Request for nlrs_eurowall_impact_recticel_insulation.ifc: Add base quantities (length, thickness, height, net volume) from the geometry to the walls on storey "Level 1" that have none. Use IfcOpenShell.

First a look at what the model holds.

```python
import ifcopenshell
import ifcopenshell.util.element
import ifcopenshell.util.unit

model = ifcopenshell.open("nlrs_eurowall_impact_recticel_insulation.ifc")
print(model.schema)
for unit_type in ("LENGTHUNIT", "AREAUNIT", "VOLUMEUNIT"):
    print(unit_type, ifcopenshell.util.unit.calculate_unit_scale(model, unit_type))
storey = next(s for s in model.by_type("IfcBuildingStorey") if s.Name == "Level 1")
walls = [e for e in ifcopenshell.util.element.get_decomposition(storey) if e.is_a("IfcWall")]
for e in sorted(walls, key=lambda e: e.id()):
    print(e.id(), e.is_a(), e.Name, list(ifcopenshell.util.element.get_psets(e, qtos_only=True)), sep=" | ")
```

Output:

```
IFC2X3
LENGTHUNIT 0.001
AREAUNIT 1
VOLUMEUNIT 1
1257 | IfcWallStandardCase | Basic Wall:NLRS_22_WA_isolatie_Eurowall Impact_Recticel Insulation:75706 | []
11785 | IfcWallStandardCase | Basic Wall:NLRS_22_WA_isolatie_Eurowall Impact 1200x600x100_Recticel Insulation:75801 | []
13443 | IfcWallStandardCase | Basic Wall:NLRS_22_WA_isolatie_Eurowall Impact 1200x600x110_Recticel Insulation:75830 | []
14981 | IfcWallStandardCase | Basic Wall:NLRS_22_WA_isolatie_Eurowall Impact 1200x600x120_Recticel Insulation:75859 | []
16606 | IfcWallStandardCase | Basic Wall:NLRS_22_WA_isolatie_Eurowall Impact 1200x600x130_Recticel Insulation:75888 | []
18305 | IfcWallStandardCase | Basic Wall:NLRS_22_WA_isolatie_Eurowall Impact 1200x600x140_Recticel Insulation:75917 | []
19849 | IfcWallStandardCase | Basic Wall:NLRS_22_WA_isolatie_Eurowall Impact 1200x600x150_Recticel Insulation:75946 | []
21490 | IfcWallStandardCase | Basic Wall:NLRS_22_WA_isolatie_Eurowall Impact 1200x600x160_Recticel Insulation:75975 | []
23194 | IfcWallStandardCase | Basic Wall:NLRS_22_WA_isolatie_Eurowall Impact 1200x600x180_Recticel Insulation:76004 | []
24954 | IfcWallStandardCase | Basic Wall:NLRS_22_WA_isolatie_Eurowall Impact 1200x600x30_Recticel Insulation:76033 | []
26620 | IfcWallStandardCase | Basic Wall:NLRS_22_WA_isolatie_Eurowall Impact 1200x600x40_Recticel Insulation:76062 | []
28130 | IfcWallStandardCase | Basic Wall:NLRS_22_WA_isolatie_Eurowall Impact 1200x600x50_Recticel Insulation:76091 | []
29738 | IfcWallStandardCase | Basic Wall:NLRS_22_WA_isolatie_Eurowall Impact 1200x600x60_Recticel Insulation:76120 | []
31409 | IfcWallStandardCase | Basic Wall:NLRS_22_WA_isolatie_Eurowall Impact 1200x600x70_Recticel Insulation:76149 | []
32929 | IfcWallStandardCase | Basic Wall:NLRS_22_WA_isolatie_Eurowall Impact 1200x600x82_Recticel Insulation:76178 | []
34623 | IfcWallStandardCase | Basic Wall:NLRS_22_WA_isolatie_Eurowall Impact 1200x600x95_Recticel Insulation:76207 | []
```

```python
import ifcopenshell
import ifcopenshell.api.pset
import ifcopenshell.geom
import ifcopenshell.util.element
import ifcopenshell.util.shape
import ifcopenshell.util.unit

model = ifcopenshell.open("nlrs_eurowall_impact_recticel_insulation.ifc")
unit_scale = ifcopenshell.util.unit.calculate_unit_scale(model)
volume_scale = ifcopenshell.util.unit.calculate_unit_scale(model, "VOLUMEUNIT")
settings = ifcopenshell.geom.settings()

storey = next(s for s in model.by_type("IfcBuildingStorey") if s.Name == "Level 1")
walls = [e for e in ifcopenshell.util.element.get_decomposition(storey) if e.is_a("IfcWall")]

for e in sorted(walls, key=lambda e: e.id()):
    if ifcopenshell.util.element.get_psets(e, qtos_only=True, should_inherit=False):
        continue
    # Geometry comes back in metres, in the element's own axes.
    shape = ifcopenshell.geom.create_shape(settings, e)
    values = {
        "Length": ifcopenshell.util.shape.get_x(shape.geometry) / unit_scale,
        "Width": ifcopenshell.util.shape.get_y(shape.geometry) / unit_scale,
        "Height": ifcopenshell.util.shape.get_z(shape.geometry) / unit_scale,
        "NetVolume": ifcopenshell.util.shape.get_volume(shape.geometry) / volume_scale,
    }
    qto = ifcopenshell.api.pset.add_qto(model, product=e, name="BaseQuantities")
    ifcopenshell.api.pset.edit_qto(model, qto=qto, properties=values)
    print(e.id(), {k: round(v, 3) for k, v in values.items()})

model.write("nlrs_eurowall_impact_recticel_insulation-out.ifc")
```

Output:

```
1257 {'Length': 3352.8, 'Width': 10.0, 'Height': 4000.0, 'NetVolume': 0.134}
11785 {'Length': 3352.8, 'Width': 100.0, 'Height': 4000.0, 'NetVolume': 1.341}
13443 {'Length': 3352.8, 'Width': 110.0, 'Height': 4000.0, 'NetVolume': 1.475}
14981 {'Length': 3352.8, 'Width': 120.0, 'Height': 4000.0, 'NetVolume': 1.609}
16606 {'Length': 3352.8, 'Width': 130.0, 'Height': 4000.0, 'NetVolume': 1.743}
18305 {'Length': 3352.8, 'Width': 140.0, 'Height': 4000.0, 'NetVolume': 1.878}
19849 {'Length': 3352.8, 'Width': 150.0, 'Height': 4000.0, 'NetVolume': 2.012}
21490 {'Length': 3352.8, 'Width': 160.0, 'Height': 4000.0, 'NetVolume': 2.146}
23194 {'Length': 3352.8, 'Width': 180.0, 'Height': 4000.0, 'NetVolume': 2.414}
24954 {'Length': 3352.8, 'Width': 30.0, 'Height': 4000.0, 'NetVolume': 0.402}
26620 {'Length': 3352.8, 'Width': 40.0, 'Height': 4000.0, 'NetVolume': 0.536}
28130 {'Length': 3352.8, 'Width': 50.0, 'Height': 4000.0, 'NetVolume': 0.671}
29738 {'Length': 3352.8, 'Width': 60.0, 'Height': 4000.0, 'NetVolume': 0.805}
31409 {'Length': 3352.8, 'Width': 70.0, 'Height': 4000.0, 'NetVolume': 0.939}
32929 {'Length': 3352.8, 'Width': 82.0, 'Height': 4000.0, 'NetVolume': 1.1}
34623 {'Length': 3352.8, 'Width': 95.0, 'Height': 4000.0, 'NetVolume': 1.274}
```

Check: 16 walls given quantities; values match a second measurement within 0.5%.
